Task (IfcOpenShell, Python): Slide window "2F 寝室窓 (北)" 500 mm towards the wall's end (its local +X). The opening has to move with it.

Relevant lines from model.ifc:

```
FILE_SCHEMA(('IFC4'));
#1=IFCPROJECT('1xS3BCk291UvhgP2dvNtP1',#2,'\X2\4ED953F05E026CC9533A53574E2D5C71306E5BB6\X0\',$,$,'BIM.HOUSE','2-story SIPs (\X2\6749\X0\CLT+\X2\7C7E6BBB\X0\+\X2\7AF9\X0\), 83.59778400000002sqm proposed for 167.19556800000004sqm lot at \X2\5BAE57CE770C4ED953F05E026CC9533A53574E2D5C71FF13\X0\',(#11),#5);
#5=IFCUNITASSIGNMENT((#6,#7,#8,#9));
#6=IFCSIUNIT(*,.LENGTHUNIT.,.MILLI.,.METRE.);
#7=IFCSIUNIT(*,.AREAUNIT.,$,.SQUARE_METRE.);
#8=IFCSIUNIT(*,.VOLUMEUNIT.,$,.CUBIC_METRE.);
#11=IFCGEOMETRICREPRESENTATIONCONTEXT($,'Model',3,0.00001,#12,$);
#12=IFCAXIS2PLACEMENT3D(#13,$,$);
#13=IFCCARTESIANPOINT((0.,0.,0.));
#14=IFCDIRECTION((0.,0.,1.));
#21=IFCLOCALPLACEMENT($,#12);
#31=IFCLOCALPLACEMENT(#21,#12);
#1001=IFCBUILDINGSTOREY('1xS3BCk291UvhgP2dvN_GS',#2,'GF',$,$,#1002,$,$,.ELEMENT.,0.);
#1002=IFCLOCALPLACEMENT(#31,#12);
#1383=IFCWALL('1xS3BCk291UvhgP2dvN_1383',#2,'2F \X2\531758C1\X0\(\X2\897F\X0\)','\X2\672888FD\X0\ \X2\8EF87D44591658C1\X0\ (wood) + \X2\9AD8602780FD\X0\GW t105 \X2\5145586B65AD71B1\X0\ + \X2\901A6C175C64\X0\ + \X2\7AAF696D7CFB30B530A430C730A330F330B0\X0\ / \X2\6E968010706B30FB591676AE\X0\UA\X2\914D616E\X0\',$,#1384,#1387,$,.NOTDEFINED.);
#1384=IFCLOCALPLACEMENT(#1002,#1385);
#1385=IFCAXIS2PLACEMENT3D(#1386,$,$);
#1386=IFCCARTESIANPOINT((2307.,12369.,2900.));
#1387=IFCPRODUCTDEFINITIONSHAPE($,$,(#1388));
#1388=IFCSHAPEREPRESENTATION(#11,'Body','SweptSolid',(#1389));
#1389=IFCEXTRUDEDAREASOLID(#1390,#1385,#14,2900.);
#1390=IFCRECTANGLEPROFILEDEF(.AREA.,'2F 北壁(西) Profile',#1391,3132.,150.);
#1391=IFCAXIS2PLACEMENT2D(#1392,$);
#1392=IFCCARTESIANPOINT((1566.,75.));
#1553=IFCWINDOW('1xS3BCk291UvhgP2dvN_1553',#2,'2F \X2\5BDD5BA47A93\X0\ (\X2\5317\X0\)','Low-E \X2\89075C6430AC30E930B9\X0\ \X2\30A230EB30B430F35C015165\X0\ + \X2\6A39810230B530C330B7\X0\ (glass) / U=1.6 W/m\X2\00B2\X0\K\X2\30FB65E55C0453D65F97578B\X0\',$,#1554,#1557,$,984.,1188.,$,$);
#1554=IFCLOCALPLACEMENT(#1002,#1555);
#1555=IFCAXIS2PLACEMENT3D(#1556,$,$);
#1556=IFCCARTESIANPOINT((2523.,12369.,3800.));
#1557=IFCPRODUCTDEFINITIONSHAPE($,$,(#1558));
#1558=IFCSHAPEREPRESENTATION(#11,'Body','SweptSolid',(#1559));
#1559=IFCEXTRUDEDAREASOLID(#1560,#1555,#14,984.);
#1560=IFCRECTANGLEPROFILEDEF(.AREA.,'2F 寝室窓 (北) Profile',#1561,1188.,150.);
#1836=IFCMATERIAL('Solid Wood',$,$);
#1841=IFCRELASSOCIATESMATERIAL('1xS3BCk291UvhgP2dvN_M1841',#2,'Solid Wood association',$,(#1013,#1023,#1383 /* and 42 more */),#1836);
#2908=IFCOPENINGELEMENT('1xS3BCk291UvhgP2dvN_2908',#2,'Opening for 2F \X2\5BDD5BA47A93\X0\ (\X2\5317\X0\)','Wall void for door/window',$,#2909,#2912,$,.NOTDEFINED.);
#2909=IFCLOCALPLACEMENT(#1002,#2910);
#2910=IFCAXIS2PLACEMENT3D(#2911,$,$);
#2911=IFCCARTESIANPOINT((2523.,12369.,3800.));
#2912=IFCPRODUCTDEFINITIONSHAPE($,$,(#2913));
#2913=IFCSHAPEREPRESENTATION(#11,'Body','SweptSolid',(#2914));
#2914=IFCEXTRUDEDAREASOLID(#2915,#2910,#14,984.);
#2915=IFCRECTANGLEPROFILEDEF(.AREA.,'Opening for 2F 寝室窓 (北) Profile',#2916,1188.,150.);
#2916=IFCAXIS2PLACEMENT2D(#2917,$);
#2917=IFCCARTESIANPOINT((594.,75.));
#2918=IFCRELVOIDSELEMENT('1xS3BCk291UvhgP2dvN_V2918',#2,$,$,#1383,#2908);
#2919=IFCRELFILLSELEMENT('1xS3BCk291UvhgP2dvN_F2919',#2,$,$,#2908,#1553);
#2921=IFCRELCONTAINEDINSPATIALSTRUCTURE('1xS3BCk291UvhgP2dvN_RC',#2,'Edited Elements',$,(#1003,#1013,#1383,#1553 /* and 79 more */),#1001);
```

```python
import ifcopenshell
import ifcopenshell.api.geometry
import ifcopenshell.util.placement
import ifcopenshell.util.unit

model = ifcopenshell.open("model.ifc")
unit_scale = ifcopenshell.util.unit.calculate_unit_scale(model)

window = model.by_guid("1xS3BCk291UvhgP2dvN_1553")
opening = window.FillsVoids[0].RelatingOpeningElement
wall = opening.VoidsElements[0].RelatingBuildingElement

wall_matrix = ifcopenshell.util.placement.get_local_placement(wall.ObjectPlacement)
shift = wall_matrix[:3, 0] * 0.5 / unit_scale
before = ifcopenshell.util.placement.get_local_placement(window.ObjectPlacement)[:3, 3].copy()

# The window is not placed relative to its opening, so move both.
for product in (opening, window):
    matrix = ifcopenshell.util.placement.get_local_placement(product.ObjectPlacement)
    matrix[:3, 3] += shift
    ifcopenshell.api.geometry.edit_object_placement(model, product=product, matrix=matrix, is_si=False)

after = ifcopenshell.util.placement.get_local_placement(window.ObjectPlacement)[:3, 3]
print("window moved by", (after - before).round(3) + 0.0)

model.write("model_edited.ifc")
```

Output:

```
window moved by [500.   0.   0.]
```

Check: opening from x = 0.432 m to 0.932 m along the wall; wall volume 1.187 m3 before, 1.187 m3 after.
